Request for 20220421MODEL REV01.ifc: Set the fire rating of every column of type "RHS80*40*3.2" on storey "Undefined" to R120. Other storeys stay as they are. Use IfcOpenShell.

First a look at what the model holds.

```python
import ifcopenshell
import ifcopenshell.util.element

model = ifcopenshell.open("20220421MODEL REV01.ifc")
print(model.schema)
storey = next(s for s in model.by_type("IfcBuildingStorey") if s.Name == "Undefined")
columns = [e for e in ifcopenshell.util.element.get_decomposition(storey) if e.is_a("IfcColumn")]
seen = {}
for e in columns:
    element_type = ifcopenshell.util.element.get_type(e)
    key = (element_type.Name if element_type != e and element_type else None, ifcopenshell.util.element.get_pset(e, "Pset_ColumnCommon", "FireRating"))
    seen[key] = seen.get(key, 0) + 1
for (name, value), count in sorted(seen.items(), key=str):
    print(count, "x", name, "|", value)
```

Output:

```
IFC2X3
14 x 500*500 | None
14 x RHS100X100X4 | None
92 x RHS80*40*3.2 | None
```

```python
import ifcopenshell
import ifcopenshell.api.pset
import ifcopenshell.util.element

model = ifcopenshell.open("20220421MODEL REV01.ifc")

storey = next(s for s in model.by_type("IfcBuildingStorey") if s.Name == "Undefined")
columns = [e for e in ifcopenshell.util.element.get_decomposition(storey) if e.is_a("IfcColumn")]

count = 0
for e in columns:
    element_type = ifcopenshell.util.element.get_type(e)
    if element_type in (None, e) or element_type.Name != "RHS80*40*3.2":
        continue
    found = ifcopenshell.util.element.get_pset(e, "Pset_ColumnCommon", should_inherit=False)
    if found:
        pset = model.by_id(found["id"])
        if len(ifcopenshell.util.element.get_elements_by_pset(pset)) > 1:
            pset = ifcopenshell.api.pset.unshare_pset(model, products=[e], pset=pset)[0]
    else:
        pset = ifcopenshell.api.pset.add_pset(model, product=e, name="Pset_ColumnCommon")
    ifcopenshell.api.pset.edit_pset(model, pset=pset, properties={"FireRating": "R120"})
    count += 1

print(count, "columns updated")

model.write("20220421MODEL REV01_edited.ifc")
```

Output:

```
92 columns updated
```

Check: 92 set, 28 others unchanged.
